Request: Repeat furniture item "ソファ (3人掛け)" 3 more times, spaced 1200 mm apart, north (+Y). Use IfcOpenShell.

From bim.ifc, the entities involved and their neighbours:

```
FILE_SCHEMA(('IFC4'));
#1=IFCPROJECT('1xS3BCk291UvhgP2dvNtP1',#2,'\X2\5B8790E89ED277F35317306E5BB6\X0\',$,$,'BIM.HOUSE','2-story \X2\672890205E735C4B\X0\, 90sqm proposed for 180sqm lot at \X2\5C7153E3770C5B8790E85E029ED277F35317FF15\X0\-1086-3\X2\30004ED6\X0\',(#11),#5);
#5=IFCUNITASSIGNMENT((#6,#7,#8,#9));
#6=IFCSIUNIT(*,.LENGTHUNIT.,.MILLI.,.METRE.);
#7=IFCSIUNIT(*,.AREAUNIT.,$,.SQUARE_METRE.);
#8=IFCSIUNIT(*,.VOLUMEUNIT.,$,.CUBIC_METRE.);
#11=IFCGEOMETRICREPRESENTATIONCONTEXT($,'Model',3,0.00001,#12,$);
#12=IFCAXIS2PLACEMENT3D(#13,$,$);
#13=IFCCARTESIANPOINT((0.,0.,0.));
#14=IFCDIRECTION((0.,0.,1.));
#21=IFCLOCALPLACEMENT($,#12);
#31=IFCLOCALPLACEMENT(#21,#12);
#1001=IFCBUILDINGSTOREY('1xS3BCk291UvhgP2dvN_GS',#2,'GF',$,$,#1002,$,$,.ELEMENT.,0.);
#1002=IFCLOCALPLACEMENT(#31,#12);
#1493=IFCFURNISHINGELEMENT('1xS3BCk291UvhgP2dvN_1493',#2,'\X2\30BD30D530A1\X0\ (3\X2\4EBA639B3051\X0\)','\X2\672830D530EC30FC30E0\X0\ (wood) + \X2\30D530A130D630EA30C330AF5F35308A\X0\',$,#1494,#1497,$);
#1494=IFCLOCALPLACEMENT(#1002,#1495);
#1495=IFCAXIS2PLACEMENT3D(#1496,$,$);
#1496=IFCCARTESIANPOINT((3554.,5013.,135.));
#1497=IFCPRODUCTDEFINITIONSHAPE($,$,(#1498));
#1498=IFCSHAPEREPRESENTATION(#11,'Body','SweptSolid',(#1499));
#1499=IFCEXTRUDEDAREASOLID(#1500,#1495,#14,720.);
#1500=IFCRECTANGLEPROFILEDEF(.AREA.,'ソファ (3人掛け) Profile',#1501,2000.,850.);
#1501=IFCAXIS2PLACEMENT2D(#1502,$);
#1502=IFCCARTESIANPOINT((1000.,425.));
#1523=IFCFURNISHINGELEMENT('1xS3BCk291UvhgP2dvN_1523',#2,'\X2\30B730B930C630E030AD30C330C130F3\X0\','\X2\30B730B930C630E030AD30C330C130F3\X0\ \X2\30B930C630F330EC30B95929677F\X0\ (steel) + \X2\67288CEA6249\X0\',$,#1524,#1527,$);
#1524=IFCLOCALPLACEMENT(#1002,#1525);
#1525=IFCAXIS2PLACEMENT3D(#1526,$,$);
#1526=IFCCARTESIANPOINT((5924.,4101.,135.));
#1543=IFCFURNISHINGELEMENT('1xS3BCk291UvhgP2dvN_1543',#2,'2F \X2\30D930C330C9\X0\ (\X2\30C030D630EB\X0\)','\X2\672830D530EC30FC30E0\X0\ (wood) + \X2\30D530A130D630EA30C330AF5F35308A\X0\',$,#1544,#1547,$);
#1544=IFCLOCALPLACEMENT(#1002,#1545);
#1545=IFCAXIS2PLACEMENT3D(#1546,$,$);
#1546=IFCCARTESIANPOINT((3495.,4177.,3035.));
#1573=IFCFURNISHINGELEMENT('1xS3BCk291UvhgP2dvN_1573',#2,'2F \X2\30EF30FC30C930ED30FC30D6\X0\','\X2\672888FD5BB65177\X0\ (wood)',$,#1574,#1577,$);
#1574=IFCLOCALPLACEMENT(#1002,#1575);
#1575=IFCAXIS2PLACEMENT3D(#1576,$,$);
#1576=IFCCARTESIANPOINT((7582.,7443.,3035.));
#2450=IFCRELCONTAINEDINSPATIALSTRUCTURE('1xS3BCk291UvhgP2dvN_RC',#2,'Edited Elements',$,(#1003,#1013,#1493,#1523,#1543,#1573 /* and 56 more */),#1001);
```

```python
import numpy as np
import ifcopenshell
import ifcopenshell.api.geometry
import ifcopenshell.api.root
import ifcopenshell.util.element
import ifcopenshell.util.placement
import ifcopenshell.util.unit

model = ifcopenshell.open("bim.ifc")
unit_scale = ifcopenshell.util.unit.calculate_unit_scale(model)


def reuse_history(source, copy):
    """copy_class also copies each property set's owner history, people and application; keep the originals."""
    for rel in copy.IsDefinedBy:
        if rel.is_a("IfcRelDefinesByProperties") and (history := rel.RelatingPropertyDefinition.OwnerHistory):
            rel.RelatingPropertyDefinition.OwnerHistory = source.OwnerHistory
            ifcopenshell.util.element.remove_deep2(model, history)


source = model.by_guid("1xS3BCk291UvhgP2dvN_1493")
base = ifcopenshell.util.placement.get_local_placement(source.ObjectPlacement)
step = np.array([0.0, 1.0, 0.0]) * 1.2 / unit_scale

for i in range(1, 4):
    copy = ifcopenshell.api.root.copy_class(model, product=source)
    copy.Representation = ifcopenshell.util.element.copy_deep(
        model, source.Representation, exclude=["IfcGeometricRepresentationContext", "IfcRepresentationMap"]
    )
    reuse_history(source, copy)
    matrix = base.copy()
    matrix[:3, 3] += i * step
    print("added at", matrix[:3, 3].round(3) + 0.0)
    ifcopenshell.api.geometry.edit_object_placement(model, product=copy, matrix=matrix, is_si=False)

model.write("bim_updated.ifc")
```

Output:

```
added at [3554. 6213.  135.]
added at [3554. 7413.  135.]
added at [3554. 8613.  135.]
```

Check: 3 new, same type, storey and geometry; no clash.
